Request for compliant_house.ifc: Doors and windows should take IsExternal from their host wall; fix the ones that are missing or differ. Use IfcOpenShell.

First a look at what the model holds.

```python
import ifcopenshell
import ifcopenshell.util.element

model = ifcopenshell.open("compliant_house.ifc")
print(model.schema)
seen = {}
for e in model.by_type("IfcDoor") + model.by_type("IfcWindow"):
    if not e.FillsVoids:
        continue
    host = e.FillsVoids[0].RelatingOpeningElement.VoidsElements[0].RelatingBuildingElement
    own = ifcopenshell.util.element.get_pset(e, f"Pset_{e.is_a()[3:].removesuffix('StandardCase')}Common", "IsExternal")
    wall = ifcopenshell.util.element.get_pset(host, "Pset_WallCommon", "IsExternal")
    seen[e.is_a(), own, wall] = seen.get((e.is_a(), own, wall), 0) + 1
for (cls, own, wall), count in sorted(seen.items(), key=str):
    print(count, cls, "IsExternal:", own, "| host wall:", wall)
```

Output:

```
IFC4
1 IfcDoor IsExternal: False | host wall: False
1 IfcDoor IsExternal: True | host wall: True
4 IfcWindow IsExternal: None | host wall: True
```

```python
import ifcopenshell
import ifcopenshell.api.pset
import ifcopenshell.util.element

model = ifcopenshell.open("compliant_house.ifc")

count = 0
for ifc_class, pset_name in (("IfcDoor", "Pset_DoorCommon"), ("IfcWindow", "Pset_WindowCommon")):
    for e in model.by_type(ifc_class):
        if not e.FillsVoids:
            continue
        host = e.FillsVoids[0].RelatingOpeningElement.VoidsElements[0].RelatingBuildingElement
        external = ifcopenshell.util.element.get_pset(host, "Pset_WallCommon", "IsExternal")
        if external is None or ifcopenshell.util.element.get_pset(e, pset_name, "IsExternal") == external:
            continue
        pset = ifcopenshell.api.pset.add_pset(model, product=e, name=pset_name)
        ifcopenshell.api.pset.edit_pset(model, pset=pset, properties={"IsExternal": external})
        count += 1

print(count, "updated")

model.write("compliant_house-out.ifc")
```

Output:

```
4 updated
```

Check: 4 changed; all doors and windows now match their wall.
